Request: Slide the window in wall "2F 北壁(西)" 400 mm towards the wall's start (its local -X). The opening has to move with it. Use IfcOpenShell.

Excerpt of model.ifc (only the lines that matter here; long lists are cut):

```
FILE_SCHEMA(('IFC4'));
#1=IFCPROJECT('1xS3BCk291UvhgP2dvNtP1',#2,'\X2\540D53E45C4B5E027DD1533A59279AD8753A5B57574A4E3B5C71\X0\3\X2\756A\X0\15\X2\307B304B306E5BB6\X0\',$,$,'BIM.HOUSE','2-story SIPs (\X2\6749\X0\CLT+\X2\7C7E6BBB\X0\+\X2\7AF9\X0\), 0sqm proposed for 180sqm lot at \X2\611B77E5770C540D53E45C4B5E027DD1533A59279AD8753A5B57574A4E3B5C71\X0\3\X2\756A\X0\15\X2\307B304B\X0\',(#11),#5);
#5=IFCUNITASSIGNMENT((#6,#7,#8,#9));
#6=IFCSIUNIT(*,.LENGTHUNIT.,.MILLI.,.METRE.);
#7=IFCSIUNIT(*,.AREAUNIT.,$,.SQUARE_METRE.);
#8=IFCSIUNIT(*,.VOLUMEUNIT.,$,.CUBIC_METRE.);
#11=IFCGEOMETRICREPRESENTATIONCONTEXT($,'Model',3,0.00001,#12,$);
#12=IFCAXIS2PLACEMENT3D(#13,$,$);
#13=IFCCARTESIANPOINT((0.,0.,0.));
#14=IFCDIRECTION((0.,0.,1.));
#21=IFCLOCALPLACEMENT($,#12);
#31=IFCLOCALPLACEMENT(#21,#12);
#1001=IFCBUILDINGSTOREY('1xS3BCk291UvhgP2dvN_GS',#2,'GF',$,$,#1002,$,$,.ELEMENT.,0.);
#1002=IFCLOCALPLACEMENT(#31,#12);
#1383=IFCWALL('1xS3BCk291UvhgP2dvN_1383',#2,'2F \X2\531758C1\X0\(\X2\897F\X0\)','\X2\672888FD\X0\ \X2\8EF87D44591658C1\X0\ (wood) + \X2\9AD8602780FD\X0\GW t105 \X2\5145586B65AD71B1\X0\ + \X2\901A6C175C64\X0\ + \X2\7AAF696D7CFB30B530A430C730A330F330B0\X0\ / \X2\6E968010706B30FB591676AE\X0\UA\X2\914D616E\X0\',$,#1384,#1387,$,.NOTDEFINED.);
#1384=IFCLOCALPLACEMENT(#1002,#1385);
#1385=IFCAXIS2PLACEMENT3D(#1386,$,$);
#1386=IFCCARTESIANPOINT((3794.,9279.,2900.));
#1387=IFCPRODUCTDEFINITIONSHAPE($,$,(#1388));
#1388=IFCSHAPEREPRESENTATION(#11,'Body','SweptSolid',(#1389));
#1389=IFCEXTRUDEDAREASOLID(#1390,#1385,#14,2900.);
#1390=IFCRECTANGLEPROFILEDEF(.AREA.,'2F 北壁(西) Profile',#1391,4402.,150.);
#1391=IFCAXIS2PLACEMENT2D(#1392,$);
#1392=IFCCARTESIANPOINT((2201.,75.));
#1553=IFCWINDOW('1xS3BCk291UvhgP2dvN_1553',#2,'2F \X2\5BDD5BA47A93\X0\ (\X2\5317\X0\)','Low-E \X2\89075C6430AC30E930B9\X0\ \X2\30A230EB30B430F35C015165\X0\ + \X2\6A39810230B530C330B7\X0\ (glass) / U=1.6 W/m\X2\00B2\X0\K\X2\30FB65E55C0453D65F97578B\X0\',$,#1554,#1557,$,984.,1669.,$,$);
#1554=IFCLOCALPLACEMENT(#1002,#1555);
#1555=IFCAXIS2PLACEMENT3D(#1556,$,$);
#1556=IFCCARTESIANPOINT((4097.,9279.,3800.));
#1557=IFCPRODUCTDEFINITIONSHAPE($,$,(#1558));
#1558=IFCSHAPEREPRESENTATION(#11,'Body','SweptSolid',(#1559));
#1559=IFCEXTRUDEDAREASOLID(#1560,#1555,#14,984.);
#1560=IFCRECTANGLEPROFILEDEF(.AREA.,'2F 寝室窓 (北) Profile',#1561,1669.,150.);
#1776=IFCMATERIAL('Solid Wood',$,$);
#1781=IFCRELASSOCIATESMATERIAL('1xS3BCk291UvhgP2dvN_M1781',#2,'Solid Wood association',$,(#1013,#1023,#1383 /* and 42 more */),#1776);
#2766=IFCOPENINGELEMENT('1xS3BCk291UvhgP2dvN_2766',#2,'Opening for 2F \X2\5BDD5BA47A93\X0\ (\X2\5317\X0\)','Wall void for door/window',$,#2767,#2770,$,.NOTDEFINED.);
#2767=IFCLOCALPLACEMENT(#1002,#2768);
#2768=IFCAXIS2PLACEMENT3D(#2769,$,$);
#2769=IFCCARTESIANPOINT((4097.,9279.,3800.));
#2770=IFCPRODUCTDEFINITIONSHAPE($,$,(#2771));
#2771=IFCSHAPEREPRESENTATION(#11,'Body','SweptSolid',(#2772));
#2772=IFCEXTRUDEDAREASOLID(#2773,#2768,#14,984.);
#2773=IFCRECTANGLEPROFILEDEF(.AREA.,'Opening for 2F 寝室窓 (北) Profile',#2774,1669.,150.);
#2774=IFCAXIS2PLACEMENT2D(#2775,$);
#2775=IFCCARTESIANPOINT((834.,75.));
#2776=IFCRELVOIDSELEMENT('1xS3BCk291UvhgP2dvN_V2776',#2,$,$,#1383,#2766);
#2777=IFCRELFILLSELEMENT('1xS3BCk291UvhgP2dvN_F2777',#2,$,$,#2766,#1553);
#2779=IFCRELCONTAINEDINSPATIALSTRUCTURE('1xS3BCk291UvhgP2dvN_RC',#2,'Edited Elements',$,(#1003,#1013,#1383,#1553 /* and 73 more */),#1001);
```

```python
import ifcopenshell
import ifcopenshell.api.geometry
import ifcopenshell.util.placement

model = ifcopenshell.open("model.ifc")

window = model.by_guid("1xS3BCk291UvhgP2dvN_1553")
opening = window.FillsVoids[0].RelatingOpeningElement
wall = opening.VoidsElements[0].RelatingBuildingElement

wall_matrix = ifcopenshell.util.placement.get_local_placement(wall.ObjectPlacement)
shift = wall_matrix[:3, 0] * -400.0
before = ifcopenshell.util.placement.get_local_placement(window.ObjectPlacement)[:3, 3].copy()

# The window is not placed relative to its opening, so move both.
for product in (opening, window):
    matrix = ifcopenshell.util.placement.get_local_placement(product.ObjectPlacement)
    matrix[:3, 3] += shift
    ifcopenshell.api.geometry.edit_object_placement(model, product=product, matrix=matrix, is_si=False)

after = ifcopenshell.util.placement.get_local_placement(window.ObjectPlacement)[:3, 3]
print("window moved by", (after - before).round(3) + 0.0)

model.write("model-out.ifc")
```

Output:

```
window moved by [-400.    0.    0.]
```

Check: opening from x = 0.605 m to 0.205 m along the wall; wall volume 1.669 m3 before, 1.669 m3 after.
